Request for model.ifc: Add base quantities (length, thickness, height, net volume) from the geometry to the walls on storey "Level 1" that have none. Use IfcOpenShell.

First a look at what the model holds.

```python
import ifcopenshell
import ifcopenshell.util.element
import ifcopenshell.util.unit

model = ifcopenshell.open("model.ifc")
print(model.schema)
for unit_type in ("LENGTHUNIT", "AREAUNIT", "VOLUMEUNIT"):
    print(unit_type, ifcopenshell.util.unit.calculate_unit_scale(model, unit_type))
storey = next(s for s in model.by_type("IfcBuildingStorey") if s.Name == "Level 1")
walls = [e for e in ifcopenshell.util.element.get_decomposition(storey) if e.is_a("IfcWall")]
for e in sorted(walls, key=lambda e: e.id()):
    print(e.id(), e.is_a(), e.Name, list(ifcopenshell.util.element.get_psets(e, qtos_only=True)), sep=" | ")
```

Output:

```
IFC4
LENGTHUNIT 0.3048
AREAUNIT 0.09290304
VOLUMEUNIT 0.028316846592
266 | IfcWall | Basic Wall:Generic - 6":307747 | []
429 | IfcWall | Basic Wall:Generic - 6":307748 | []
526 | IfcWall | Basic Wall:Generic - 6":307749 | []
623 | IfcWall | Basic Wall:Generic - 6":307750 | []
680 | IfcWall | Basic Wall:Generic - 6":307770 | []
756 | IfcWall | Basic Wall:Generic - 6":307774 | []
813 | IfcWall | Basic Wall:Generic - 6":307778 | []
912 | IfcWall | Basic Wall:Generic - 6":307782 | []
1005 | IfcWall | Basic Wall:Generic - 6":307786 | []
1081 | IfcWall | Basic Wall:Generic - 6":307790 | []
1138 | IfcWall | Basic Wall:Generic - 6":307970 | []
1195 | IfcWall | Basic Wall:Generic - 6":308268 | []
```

```python
import ifcopenshell
import ifcopenshell.api.pset
import ifcopenshell.geom
import ifcopenshell.util.element
import ifcopenshell.util.shape
import ifcopenshell.util.unit

model = ifcopenshell.open("model.ifc")
unit_scale = ifcopenshell.util.unit.calculate_unit_scale(model)
volume_scale = ifcopenshell.util.unit.calculate_unit_scale(model, "VOLUMEUNIT")
settings = ifcopenshell.geom.settings()

storey = next(s for s in model.by_type("IfcBuildingStorey") if s.Name == "Level 1")
walls = [e for e in ifcopenshell.util.element.get_decomposition(storey) if e.is_a("IfcWall")]

for e in sorted(walls, key=lambda e: e.id()):
    if ifcopenshell.util.element.get_psets(e, qtos_only=True, should_inherit=False):
        continue
    # Geometry comes back in metres, in the element's own axes.
    shape = ifcopenshell.geom.create_shape(settings, e)
    values = {
        "Length": ifcopenshell.util.shape.get_x(shape.geometry) / unit_scale,
        "Width": ifcopenshell.util.shape.get_y(shape.geometry) / unit_scale,
        "Height": ifcopenshell.util.shape.get_z(shape.geometry) / unit_scale,
        "NetVolume": ifcopenshell.util.shape.get_volume(shape.geometry) / volume_scale,
    }
    qto = ifcopenshell.api.pset.add_qto(model, product=e, name="Qto_WallBaseQuantities")
    ifcopenshell.api.pset.edit_qto(model, qto=qto, properties=values)
    print(e.id(), {k: round(v, 3) for k, v in values.items()})

model.write("model-out.ifc")
```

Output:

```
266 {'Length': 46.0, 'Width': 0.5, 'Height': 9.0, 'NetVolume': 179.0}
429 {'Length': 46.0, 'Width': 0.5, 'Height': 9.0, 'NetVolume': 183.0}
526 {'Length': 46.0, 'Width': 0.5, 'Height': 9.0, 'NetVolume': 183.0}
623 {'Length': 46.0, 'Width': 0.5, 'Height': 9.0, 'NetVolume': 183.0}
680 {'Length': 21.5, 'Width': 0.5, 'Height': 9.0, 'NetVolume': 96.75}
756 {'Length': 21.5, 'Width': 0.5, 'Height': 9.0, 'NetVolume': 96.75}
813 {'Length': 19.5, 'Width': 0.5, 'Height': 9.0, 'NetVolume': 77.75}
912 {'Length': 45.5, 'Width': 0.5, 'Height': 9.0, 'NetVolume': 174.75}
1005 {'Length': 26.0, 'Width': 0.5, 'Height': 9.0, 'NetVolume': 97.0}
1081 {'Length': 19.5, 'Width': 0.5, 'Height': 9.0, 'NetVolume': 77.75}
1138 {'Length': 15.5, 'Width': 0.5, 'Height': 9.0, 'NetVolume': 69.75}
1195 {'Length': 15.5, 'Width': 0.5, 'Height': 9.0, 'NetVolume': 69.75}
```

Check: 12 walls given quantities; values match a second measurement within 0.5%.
